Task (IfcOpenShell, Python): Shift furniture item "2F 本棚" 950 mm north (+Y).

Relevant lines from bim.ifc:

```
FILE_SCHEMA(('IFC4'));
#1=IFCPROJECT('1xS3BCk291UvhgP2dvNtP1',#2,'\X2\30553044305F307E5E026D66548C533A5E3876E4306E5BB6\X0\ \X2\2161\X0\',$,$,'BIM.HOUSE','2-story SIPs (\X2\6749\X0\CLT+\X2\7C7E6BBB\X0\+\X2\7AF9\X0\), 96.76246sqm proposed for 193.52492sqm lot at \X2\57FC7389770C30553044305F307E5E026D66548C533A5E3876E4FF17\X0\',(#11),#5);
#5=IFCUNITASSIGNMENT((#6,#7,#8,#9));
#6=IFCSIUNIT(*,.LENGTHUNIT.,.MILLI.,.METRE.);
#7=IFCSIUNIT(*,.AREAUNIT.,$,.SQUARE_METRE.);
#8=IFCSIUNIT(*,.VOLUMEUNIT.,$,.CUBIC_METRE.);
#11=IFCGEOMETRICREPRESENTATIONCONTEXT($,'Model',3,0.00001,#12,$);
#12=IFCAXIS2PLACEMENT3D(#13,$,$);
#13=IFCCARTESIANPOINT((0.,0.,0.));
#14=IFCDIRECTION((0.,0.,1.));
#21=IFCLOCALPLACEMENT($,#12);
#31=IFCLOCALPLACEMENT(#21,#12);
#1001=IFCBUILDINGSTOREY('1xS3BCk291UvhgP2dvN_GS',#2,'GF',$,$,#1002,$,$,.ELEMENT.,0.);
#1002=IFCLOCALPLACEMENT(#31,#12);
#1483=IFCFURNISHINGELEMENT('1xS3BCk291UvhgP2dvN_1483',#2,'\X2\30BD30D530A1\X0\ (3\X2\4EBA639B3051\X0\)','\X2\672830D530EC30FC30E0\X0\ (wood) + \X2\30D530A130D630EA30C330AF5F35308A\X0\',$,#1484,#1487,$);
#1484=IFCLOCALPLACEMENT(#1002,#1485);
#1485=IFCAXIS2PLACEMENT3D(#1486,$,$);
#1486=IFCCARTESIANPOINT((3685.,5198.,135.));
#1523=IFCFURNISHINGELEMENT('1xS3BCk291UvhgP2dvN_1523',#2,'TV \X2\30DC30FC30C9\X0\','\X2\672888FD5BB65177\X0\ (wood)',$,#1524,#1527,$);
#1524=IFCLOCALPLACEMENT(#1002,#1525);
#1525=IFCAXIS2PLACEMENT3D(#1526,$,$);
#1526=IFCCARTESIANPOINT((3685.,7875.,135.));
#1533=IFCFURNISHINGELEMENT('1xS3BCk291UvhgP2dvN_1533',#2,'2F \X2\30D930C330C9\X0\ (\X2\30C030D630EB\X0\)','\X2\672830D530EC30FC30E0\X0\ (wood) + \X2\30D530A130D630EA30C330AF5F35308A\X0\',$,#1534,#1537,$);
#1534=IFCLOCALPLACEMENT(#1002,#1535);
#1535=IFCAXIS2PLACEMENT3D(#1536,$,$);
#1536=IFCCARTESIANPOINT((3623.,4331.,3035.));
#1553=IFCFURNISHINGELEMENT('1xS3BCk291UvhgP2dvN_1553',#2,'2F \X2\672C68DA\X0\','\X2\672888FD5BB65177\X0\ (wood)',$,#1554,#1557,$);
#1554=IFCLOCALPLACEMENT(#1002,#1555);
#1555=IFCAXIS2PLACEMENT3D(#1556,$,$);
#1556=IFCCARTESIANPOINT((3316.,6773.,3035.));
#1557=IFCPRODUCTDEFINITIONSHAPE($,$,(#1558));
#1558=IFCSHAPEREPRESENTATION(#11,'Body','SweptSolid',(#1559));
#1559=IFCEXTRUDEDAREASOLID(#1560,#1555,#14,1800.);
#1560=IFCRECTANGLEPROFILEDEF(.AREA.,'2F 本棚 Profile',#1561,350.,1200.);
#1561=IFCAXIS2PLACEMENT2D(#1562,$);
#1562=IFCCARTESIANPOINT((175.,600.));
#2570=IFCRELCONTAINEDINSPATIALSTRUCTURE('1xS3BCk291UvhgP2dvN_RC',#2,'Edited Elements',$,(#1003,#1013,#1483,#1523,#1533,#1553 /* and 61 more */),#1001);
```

```python
import ifcopenshell
import ifcopenshell.api.geometry
import ifcopenshell.util.placement
import ifcopenshell.util.unit

model = ifcopenshell.open("bim.ifc")
unit_scale = ifcopenshell.util.unit.calculate_unit_scale(model)

item = model.by_guid("1xS3BCk291UvhgP2dvN_1553")
matrix = ifcopenshell.util.placement.get_local_placement(item.ObjectPlacement)
matrix[1, 3] += 0.95 / unit_scale
ifcopenshell.api.geometry.edit_object_placement(model, product=item, matrix=matrix, is_si=False)

print(ifcopenshell.util.placement.get_local_placement(item.ObjectPlacement).round(3) + 0.0)

model.write("bim_edited.ifc")
```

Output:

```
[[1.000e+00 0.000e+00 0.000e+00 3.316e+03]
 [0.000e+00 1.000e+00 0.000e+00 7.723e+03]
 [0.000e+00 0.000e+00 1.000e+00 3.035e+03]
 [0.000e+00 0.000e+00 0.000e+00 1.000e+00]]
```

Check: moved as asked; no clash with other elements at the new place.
